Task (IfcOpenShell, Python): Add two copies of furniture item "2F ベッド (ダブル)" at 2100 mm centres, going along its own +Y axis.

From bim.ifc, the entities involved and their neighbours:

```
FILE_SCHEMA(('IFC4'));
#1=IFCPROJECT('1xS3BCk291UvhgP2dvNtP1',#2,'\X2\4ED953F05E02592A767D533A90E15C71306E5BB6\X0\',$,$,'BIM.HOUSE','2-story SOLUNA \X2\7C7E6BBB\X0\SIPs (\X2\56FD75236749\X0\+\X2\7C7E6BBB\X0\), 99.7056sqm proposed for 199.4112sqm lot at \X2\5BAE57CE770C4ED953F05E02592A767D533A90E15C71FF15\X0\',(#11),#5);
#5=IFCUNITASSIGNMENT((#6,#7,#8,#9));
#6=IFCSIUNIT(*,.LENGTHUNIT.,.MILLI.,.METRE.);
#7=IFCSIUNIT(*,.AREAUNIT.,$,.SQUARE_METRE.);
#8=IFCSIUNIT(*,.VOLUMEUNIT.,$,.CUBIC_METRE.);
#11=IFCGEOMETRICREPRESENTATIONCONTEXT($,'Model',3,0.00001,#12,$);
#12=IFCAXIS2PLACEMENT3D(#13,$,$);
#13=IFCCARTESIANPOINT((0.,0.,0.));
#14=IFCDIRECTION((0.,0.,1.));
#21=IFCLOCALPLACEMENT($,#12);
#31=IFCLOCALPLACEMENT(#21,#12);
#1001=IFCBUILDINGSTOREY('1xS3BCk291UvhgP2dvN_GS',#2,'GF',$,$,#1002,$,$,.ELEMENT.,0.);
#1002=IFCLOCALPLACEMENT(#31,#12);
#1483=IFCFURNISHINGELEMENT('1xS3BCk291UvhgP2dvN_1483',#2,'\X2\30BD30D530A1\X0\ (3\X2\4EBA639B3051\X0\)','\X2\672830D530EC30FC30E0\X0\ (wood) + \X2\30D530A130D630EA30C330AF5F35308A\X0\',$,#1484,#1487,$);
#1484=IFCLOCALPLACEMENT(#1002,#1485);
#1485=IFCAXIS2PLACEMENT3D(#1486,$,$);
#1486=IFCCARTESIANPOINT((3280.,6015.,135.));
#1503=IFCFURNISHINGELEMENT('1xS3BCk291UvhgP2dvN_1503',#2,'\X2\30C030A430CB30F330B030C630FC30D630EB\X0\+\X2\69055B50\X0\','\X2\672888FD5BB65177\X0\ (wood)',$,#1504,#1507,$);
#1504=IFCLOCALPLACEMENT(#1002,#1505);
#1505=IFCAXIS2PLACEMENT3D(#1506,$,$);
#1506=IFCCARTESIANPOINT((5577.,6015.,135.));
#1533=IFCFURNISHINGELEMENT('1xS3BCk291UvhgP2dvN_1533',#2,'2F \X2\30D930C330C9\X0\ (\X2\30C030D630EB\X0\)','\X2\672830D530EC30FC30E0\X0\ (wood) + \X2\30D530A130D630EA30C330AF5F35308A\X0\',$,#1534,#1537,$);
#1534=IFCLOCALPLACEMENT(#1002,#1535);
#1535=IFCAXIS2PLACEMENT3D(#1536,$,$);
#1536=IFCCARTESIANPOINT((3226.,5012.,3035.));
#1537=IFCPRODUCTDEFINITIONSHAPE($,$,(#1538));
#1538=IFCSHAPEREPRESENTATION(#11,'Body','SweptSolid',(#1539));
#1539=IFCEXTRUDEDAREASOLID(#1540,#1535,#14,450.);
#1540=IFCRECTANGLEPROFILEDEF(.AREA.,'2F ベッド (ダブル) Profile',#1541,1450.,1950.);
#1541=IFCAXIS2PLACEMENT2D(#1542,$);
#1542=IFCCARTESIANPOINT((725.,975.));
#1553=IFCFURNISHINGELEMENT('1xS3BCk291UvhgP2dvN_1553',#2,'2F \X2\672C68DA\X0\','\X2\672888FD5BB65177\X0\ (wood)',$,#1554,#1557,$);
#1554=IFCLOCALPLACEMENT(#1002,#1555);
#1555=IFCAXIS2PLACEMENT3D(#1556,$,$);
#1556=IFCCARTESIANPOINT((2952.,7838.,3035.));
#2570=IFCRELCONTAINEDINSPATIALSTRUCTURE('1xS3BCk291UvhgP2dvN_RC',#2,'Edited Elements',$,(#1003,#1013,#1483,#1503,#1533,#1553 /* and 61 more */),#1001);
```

```python
import ifcopenshell
import ifcopenshell.api.geometry
import ifcopenshell.api.root
import ifcopenshell.util.element
import ifcopenshell.util.placement

model = ifcopenshell.open("bim.ifc")


def reuse_history(source, copy):
    """copy_class also copies each property set's owner history, people and application; keep the originals."""
    for rel in copy.IsDefinedBy:
        if rel.is_a("IfcRelDefinesByProperties") and (history := rel.RelatingPropertyDefinition.OwnerHistory):
            rel.RelatingPropertyDefinition.OwnerHistory = source.OwnerHistory
            ifcopenshell.util.element.remove_deep2(model, history)


source = model.by_id(1533)
base = ifcopenshell.util.placement.get_local_placement(source.ObjectPlacement)
step = base[:3, 1] * 2100.0

for i in range(1, 3):
    copy = ifcopenshell.api.root.copy_class(model, product=source)
    copy.Representation = ifcopenshell.util.element.copy_deep(
        model, source.Representation, exclude=["IfcGeometricRepresentationContext", "IfcRepresentationMap"]
    )
    reuse_history(source, copy)
    matrix = base.copy()
    matrix[:3, 3] += i * step
    print("added at", matrix[:3, 3].round(3) + 0.0)
    ifcopenshell.api.geometry.edit_object_placement(model, product=copy, matrix=matrix, is_si=False)

model.write("bim_edited.ifc")
```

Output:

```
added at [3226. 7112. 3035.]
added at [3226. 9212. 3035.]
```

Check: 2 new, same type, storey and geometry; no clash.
